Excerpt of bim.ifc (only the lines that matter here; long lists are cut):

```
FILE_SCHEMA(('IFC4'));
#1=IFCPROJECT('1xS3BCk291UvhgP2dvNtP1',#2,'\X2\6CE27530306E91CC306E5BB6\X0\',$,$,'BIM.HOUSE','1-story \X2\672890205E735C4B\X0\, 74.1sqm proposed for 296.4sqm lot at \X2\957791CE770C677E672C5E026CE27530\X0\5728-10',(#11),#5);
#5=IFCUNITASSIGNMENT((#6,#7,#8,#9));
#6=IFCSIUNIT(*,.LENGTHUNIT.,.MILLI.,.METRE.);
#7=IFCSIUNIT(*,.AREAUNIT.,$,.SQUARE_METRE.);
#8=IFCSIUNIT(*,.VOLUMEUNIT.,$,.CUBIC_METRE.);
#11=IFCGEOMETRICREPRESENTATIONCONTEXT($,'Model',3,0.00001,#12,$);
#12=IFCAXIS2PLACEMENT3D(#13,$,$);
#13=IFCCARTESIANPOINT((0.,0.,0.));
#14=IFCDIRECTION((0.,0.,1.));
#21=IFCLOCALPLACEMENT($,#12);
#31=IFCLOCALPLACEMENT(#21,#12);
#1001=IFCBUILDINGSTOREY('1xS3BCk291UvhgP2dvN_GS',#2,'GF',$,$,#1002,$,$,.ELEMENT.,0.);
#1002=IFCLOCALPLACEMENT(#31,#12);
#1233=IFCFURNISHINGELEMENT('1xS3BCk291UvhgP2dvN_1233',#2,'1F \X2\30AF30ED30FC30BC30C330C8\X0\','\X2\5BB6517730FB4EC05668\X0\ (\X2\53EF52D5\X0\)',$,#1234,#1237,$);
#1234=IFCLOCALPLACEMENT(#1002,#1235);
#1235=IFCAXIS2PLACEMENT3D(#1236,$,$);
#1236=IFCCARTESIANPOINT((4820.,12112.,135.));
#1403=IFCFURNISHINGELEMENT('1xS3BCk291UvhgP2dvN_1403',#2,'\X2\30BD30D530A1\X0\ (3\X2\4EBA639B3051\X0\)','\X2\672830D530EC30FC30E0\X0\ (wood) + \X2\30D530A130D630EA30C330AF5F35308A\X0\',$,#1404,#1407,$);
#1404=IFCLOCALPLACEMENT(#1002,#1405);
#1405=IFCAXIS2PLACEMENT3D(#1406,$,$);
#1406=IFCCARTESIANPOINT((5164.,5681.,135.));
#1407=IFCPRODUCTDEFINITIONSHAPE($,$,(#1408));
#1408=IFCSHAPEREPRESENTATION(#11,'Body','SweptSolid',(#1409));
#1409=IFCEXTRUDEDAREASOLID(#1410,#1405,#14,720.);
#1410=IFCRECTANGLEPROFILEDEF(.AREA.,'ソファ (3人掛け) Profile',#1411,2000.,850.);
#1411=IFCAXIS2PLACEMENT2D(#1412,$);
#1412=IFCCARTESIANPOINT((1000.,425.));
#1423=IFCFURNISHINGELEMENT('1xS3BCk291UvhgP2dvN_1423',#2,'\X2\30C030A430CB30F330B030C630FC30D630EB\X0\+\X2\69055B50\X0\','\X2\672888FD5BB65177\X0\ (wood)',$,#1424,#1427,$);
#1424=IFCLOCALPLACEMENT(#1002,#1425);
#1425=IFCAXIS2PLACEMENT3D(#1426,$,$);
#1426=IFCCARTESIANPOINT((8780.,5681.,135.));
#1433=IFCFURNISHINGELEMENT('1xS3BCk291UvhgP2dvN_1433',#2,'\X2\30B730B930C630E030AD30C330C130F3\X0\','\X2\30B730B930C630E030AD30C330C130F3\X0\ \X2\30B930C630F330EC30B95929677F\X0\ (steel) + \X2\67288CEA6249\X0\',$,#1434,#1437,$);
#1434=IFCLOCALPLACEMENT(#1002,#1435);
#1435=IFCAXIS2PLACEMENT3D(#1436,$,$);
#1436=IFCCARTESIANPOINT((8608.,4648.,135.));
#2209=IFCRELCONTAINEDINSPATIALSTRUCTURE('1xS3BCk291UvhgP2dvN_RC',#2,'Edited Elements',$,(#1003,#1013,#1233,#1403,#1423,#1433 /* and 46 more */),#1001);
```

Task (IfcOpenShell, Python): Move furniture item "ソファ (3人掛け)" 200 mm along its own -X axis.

```python
import ifcopenshell
import ifcopenshell.api.geometry
import ifcopenshell.util.placement
import ifcopenshell.util.unit

model = ifcopenshell.open("bim.ifc")
unit_scale = ifcopenshell.util.unit.calculate_unit_scale(model)

item = model.by_id(1403)
matrix = ifcopenshell.util.placement.get_local_placement(item.ObjectPlacement)
matrix[:3, 3] -= matrix[:3, 0] * 0.2 / unit_scale
ifcopenshell.api.geometry.edit_object_placement(model, product=item, matrix=matrix, is_si=False)

print(ifcopenshell.util.placement.get_local_placement(item.ObjectPlacement).round(3) + 0.0)

model.write("bim_updated.ifc")
```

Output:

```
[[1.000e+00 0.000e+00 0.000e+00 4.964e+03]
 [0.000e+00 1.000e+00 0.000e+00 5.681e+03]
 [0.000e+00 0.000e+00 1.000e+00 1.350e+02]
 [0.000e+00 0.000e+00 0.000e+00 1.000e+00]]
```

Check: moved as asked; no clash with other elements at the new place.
